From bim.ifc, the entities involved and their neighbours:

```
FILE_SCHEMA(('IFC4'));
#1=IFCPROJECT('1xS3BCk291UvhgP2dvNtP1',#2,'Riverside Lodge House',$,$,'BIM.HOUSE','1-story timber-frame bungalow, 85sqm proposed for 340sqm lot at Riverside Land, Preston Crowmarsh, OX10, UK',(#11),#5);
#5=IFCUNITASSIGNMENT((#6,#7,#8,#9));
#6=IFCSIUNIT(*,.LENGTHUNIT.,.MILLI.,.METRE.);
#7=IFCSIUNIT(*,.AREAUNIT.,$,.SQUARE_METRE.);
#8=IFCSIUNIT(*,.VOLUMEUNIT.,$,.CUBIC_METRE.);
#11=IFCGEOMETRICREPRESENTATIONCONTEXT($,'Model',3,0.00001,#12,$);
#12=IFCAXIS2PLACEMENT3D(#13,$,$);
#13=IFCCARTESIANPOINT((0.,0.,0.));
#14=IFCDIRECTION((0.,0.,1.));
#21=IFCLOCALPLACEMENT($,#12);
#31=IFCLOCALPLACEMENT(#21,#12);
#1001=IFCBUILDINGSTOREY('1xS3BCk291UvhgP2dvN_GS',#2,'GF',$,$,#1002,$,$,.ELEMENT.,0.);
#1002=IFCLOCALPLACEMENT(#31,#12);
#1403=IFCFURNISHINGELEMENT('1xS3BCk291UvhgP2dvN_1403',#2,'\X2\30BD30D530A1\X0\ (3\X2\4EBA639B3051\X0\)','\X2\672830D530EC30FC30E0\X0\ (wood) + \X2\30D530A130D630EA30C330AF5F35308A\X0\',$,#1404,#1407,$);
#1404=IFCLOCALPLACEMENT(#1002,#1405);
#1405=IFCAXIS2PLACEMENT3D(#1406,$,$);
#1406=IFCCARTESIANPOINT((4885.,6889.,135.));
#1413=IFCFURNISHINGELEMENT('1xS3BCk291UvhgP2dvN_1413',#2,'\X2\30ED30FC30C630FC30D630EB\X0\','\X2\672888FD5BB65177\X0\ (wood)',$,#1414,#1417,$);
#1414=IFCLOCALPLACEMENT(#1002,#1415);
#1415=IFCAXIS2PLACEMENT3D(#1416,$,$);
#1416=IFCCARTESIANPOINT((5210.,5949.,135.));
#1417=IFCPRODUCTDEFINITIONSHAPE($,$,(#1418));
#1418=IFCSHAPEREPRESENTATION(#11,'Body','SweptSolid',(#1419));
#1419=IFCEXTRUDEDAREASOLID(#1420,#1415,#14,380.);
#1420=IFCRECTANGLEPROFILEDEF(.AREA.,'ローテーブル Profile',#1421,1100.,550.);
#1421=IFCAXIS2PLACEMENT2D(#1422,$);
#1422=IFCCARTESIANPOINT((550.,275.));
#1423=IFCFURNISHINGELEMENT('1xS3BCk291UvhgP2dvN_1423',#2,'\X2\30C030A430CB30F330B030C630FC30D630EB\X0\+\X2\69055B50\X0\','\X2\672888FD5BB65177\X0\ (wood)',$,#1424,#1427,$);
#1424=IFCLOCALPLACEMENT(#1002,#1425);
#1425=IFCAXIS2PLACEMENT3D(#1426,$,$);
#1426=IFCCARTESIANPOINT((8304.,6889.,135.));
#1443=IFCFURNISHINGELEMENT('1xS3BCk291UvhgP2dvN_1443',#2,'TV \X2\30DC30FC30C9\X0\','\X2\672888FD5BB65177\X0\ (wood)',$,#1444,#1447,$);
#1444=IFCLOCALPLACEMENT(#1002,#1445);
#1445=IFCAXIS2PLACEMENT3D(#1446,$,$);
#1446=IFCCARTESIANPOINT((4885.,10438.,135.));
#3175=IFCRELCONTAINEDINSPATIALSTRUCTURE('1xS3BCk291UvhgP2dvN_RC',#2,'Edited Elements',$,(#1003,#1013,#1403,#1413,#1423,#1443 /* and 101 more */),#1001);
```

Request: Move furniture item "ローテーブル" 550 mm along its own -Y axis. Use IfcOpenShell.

```python
import ifcopenshell
import ifcopenshell.api.geometry
import ifcopenshell.util.placement
import ifcopenshell.util.unit

model = ifcopenshell.open("bim.ifc")
unit_scale = ifcopenshell.util.unit.calculate_unit_scale(model)

item = model.by_guid("1xS3BCk291UvhgP2dvN_1413")
matrix = ifcopenshell.util.placement.get_local_placement(item.ObjectPlacement)
matrix[:3, 3] -= matrix[:3, 1] * 0.55 / unit_scale
ifcopenshell.api.geometry.edit_object_placement(model, product=item, matrix=matrix, is_si=False)

print(ifcopenshell.util.placement.get_local_placement(item.ObjectPlacement).round(3) + 0.0)

model.write("bim_rev.ifc")
```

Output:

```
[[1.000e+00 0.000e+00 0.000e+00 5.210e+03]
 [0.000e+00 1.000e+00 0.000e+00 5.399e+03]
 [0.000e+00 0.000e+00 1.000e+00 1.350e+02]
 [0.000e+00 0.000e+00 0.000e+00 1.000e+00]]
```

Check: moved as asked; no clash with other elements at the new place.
